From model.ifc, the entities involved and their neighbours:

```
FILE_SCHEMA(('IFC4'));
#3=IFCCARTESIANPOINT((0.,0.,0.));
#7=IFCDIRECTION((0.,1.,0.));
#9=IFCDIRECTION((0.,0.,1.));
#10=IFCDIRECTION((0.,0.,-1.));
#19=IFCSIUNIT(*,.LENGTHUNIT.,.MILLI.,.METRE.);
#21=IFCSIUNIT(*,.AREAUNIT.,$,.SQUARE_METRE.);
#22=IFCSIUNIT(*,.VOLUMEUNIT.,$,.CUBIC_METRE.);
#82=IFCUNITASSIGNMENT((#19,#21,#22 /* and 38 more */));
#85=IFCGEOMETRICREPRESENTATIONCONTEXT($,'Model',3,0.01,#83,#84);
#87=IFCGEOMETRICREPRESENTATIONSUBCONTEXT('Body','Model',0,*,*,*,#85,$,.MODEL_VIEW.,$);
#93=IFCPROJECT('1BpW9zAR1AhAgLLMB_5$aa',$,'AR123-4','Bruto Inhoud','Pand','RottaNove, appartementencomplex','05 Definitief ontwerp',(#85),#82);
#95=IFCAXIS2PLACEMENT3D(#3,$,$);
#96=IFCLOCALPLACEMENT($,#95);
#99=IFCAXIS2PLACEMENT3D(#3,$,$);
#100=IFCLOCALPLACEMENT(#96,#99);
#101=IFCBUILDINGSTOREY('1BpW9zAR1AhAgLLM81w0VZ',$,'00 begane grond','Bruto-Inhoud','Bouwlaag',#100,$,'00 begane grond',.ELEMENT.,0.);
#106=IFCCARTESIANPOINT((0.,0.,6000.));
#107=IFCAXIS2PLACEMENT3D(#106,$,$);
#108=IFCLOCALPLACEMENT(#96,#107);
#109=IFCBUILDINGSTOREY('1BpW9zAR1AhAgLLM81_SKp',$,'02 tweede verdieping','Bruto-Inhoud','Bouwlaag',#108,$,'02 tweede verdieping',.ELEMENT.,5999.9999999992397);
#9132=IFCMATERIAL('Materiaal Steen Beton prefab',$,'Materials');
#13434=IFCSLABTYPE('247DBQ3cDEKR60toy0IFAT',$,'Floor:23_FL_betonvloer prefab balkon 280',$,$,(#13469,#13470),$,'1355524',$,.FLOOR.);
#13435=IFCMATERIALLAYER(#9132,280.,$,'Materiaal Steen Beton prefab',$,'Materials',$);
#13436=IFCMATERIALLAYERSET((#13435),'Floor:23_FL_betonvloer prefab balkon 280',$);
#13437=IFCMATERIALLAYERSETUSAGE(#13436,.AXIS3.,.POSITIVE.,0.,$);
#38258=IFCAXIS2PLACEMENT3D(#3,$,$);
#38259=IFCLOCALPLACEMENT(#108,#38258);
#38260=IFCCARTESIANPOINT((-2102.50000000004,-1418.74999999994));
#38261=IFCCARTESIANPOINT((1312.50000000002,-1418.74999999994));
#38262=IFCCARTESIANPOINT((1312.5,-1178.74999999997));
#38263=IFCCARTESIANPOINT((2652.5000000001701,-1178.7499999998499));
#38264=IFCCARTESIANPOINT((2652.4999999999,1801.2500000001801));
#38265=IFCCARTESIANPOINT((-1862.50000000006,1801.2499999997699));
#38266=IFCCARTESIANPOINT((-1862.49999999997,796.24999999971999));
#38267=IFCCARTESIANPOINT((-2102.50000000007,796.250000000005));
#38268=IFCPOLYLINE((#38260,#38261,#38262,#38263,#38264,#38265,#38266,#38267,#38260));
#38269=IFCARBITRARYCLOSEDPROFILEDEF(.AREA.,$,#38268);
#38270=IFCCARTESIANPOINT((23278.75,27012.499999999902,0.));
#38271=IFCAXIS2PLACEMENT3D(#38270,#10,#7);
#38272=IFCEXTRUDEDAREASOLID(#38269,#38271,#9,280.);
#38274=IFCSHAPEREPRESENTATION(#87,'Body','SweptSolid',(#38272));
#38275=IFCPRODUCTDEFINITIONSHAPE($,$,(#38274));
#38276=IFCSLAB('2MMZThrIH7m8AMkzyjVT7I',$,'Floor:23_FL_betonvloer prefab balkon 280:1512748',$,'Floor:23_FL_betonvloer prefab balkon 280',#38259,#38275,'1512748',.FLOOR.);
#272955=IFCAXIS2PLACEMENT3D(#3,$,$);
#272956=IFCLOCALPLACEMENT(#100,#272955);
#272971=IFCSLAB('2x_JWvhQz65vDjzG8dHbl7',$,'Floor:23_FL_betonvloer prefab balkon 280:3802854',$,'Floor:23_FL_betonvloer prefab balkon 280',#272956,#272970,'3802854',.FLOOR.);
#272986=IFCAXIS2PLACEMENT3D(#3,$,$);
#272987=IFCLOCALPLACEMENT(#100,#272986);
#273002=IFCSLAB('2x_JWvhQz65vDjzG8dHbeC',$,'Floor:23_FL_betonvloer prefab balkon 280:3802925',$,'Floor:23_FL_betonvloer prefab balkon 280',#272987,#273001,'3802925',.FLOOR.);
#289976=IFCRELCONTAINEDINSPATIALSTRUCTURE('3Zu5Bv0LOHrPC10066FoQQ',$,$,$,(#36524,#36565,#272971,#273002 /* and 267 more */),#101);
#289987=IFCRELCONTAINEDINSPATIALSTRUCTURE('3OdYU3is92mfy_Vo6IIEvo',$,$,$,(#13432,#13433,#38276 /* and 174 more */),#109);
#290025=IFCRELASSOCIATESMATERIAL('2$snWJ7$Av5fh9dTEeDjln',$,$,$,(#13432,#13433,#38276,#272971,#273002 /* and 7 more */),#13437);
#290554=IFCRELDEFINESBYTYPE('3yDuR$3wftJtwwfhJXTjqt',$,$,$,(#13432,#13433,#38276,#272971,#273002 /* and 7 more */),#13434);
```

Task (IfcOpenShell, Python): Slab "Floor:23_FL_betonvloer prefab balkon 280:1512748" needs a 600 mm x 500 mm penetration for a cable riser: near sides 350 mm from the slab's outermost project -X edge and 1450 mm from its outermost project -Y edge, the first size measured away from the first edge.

```python
import numpy as np
import ifcopenshell
import ifcopenshell.api.feature
import ifcopenshell.api.geometry
import ifcopenshell.api.root
import ifcopenshell.geom
import ifcopenshell.util.placement
import ifcopenshell.util.representation
import ifcopenshell.util.shape
import ifcopenshell.util.unit

model = ifcopenshell.open("model.ifc")
unit_scale = ifcopenshell.util.unit.calculate_unit_scale(model)
settings = ifcopenshell.geom.settings()


def volume(element):
    """Net volume in cubic metres, openings subtracted."""
    shape = ifcopenshell.geom.create_shape(settings, element)
    return ifcopenshell.util.shape.get_volume(shape.geometry)


slab = model.by_id(38276)
before = volume(slab)

# Extent in the slab's own axes, in metres. The edges named are its -X and -Y sides.
slab_shape = ifcopenshell.geom.create_shape(settings, slab)
vertices = ifcopenshell.util.shape.get_vertices(slab_shape.geometry)
x_min, y_min, bottom = vertices.min(axis=0)
top = vertices[:, 2].max()

opening = ifcopenshell.api.root.create_entity(model, ifc_class="IfcOpeningElement", name="Cable riser opening", predefined_type="OPENING")
context = ifcopenshell.util.representation.get_context(model, "Model", "Body", "MODEL_VIEW")
width, depth = 0.6, 0.5
outline = [(0.0, 0.0), (width, 0.0), (width, depth), (0.0, depth), (0.0, 0.0)]
# Overshoot both faces by 50 mm so the cut is clean.
shape = ifcopenshell.api.geometry.add_slab_representation(
    model, context=context, depth=top - bottom + 0.1, polyline=outline
)
ifcopenshell.api.geometry.assign_representation(model, product=opening, representation=shape)

matrix = ifcopenshell.util.placement.get_local_placement(slab.ObjectPlacement)
matrix[:, 3] = matrix @ np.append(np.array([x_min + 0.35, y_min + 1.45, bottom - 0.05]) / unit_scale, 1.0)
ifcopenshell.api.geometry.edit_object_placement(model, product=opening, matrix=matrix, is_si=False)
ifcopenshell.api.feature.add_feature(model, feature=opening, element=slab)

after = volume(slab)

print(f"slab volume {before:.3f} -> {after:.3f} m3")

model.write("model_updated.ifc")
```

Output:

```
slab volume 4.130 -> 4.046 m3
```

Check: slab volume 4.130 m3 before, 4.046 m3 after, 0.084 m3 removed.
